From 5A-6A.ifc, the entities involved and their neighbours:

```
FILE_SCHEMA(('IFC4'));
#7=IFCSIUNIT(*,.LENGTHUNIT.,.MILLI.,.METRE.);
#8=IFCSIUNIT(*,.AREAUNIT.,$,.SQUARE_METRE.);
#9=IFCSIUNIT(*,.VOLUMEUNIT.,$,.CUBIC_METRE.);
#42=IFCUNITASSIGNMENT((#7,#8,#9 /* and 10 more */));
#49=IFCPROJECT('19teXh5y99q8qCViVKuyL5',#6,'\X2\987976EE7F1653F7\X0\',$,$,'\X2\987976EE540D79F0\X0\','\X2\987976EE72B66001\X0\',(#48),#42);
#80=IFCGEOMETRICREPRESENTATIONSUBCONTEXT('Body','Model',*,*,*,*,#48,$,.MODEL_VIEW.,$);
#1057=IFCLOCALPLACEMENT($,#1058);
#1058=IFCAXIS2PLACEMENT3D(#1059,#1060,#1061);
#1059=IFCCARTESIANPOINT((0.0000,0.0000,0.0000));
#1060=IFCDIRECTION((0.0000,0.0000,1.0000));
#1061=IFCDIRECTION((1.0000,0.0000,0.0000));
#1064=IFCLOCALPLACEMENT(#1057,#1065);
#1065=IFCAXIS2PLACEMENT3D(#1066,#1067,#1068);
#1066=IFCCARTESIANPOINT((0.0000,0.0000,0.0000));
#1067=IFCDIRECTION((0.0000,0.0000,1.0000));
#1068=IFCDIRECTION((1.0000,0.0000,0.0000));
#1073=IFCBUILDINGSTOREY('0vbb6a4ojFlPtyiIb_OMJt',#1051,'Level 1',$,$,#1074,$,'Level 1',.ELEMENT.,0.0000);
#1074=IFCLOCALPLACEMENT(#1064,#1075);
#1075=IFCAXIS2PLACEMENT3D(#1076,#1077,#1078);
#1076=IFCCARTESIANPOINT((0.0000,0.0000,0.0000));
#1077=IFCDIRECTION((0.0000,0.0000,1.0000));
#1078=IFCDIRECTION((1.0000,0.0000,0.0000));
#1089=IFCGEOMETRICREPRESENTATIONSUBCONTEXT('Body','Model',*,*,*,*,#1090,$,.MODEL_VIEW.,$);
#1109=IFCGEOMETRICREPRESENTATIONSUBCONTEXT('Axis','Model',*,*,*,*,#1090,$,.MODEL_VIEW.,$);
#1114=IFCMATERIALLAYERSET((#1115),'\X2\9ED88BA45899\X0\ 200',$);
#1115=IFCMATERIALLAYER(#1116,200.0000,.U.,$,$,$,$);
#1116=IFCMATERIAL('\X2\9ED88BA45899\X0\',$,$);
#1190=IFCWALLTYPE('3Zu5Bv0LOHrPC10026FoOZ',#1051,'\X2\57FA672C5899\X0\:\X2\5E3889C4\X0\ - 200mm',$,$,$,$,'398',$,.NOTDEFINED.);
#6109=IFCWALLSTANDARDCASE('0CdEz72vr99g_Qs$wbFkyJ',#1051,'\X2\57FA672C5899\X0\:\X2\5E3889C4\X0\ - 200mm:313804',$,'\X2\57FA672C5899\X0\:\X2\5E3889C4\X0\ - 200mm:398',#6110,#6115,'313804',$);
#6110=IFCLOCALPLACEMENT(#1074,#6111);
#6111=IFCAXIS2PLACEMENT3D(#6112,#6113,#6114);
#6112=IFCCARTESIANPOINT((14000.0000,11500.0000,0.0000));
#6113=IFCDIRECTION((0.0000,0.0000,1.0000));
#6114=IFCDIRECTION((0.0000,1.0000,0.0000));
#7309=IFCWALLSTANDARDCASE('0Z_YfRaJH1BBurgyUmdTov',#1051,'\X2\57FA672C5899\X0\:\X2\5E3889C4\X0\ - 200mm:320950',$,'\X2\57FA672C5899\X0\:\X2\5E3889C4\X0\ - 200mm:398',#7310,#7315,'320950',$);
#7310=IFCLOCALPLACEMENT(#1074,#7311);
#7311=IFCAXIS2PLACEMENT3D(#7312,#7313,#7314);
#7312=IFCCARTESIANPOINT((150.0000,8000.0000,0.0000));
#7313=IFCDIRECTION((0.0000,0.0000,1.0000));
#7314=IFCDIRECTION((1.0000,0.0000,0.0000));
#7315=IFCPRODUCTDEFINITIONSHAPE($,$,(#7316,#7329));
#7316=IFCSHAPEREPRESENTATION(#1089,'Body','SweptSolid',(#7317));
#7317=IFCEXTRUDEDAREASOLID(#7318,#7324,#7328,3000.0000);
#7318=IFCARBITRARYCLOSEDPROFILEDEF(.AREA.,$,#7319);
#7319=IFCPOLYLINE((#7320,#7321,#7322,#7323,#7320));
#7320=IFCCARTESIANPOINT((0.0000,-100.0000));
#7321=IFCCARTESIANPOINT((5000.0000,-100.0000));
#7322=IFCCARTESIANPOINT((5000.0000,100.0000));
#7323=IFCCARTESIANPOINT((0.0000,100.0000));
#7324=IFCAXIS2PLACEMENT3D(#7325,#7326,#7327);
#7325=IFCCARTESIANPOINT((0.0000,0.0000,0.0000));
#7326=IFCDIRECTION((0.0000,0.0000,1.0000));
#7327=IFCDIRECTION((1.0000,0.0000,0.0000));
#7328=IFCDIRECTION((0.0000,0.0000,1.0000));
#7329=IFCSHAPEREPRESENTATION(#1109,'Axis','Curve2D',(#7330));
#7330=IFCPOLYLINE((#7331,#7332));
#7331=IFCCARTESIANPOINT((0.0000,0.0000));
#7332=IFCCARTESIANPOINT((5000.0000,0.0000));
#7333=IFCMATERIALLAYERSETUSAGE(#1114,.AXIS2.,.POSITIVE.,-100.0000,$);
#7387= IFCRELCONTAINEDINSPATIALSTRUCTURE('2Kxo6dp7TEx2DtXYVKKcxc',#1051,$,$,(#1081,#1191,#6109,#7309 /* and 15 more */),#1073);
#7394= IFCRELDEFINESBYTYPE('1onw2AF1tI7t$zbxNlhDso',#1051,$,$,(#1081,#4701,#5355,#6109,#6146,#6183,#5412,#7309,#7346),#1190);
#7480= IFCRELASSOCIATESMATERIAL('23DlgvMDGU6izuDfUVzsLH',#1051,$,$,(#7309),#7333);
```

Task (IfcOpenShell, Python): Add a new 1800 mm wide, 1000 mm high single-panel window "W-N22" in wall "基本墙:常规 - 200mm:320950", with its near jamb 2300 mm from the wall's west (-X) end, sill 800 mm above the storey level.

```python
import numpy as np
import ifcopenshell
import ifcopenshell.api.feature
import ifcopenshell.api.geometry
import ifcopenshell.api.root
import ifcopenshell.api.spatial
import ifcopenshell.geom
import ifcopenshell.util.element
import ifcopenshell.util.placement
import ifcopenshell.util.representation
import ifcopenshell.util.shape
import ifcopenshell.util.unit

model = ifcopenshell.open("5A-6A.ifc")
unit_scale = ifcopenshell.util.unit.calculate_unit_scale(model)
settings = ifcopenshell.geom.settings()


def volume(element):
    """Net volume in cubic metres, openings subtracted."""
    shape = ifcopenshell.geom.create_shape(settings, element)
    return ifcopenshell.util.shape.get_volume(shape.geometry)


wall = model.by_guid("0Z_YfRaJH1BBurgyUmdTov")
storey = ifcopenshell.util.element.get_container(wall, ifc_class="IfcBuildingStorey")
context = ifcopenshell.util.representation.get_context(model, "Model", "Body", "MODEL_VIEW")
before = volume(wall)

width, height, from_end, sill = 1.8, 1, 2.3, 0.8  # metres

# The wall runs along its own X axis, and the end named is its -X end.
wall_shape = ifcopenshell.geom.create_shape(settings, wall)
x, y, z = ifcopenshell.util.shape.get_vertices(wall_shape.geometry).T
start = x.min() + from_end
face, thickness = float(y.min()), float(y.max() - y.min())
wall_matrix = ifcopenshell.util.placement.get_local_placement(wall.ObjectPlacement)
level = ifcopenshell.util.placement.get_local_placement(storey.ObjectPlacement)[2, 3]


def in_wall(x, y):
    """Placement at x, y metres in the wall's axes, at sill height."""
    matrix = wall_matrix.copy()
    matrix[:, 3] = wall_matrix @ np.array([x / unit_scale, y / unit_scale, 0.0, 1.0])
    matrix[2, 3] = level + sill / unit_scale
    return matrix


# Opening: a box that overshoots both wall faces by 50 mm.
opening = ifcopenshell.api.root.create_entity(model, ifc_class="IfcOpeningElement", predefined_type="OPENING")
box = ifcopenshell.api.geometry.add_wall_representation(
    model, context=context, length=width, height=height, thickness=thickness + 0.1
)
ifcopenshell.api.geometry.assign_representation(model, product=opening, representation=box)
ifcopenshell.api.geometry.edit_object_placement(model, product=opening, matrix=in_wall(start, face - 0.05), is_si=False)
ifcopenshell.api.feature.add_feature(model, feature=opening, element=wall)

window = ifcopenshell.api.root.create_entity(model, ifc_class="IfcWindow", name="W-N22", predefined_type="WINDOW")
window.OverallWidth, window.OverallHeight = width / unit_scale, height / unit_scale
window.PartitioningType = "SINGLE_PANEL"
body = ifcopenshell.api.geometry.add_window_representation(
    model,
    context=context,
    overall_width=window.OverallWidth,
    overall_height=window.OverallHeight,
    partition_type="SINGLE_PANEL",
)
ifcopenshell.api.geometry.assign_representation(model, product=window, representation=body)
ifcopenshell.api.spatial.assign_container(model, products=[window], relating_structure=storey)
ifcopenshell.api.feature.add_filling(model, opening=opening, element=window)

# Centre the window in the wall's thickness.
ifcopenshell.api.geometry.edit_object_placement(model, product=window, matrix=in_wall(start, face), is_si=False)
window_shape = ifcopenshell.geom.create_shape(settings, window)
depth = ifcopenshell.util.shape.get_vertices(window_shape.geometry)[:, 1]
offset = face + thickness / 2 - (depth.min() + depth.max()) / 2
ifcopenshell.api.geometry.edit_object_placement(model, product=window, matrix=in_wall(start, offset), is_si=False)

after = volume(wall)

print(f"wall volume {before:.3f} -> {after:.3f} m3")

model.write("5A-6A_rev.ifc")
```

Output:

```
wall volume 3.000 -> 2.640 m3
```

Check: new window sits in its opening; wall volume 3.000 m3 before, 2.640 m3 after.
